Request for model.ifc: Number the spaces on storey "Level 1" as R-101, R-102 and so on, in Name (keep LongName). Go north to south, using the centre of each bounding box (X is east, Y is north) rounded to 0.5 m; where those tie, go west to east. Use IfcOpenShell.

First a look at what the model holds.

```python
import ifcopenshell
import ifcopenshell.util.element
import ifcopenshell.util.placement

model = ifcopenshell.open("model.ifc")
print(model.schema)
storey = next(s for s in model.by_type("IfcBuildingStorey") if s.Name == "Level 1")
spaces = [e for e in ifcopenshell.util.element.get_decomposition(storey) if e.is_a("IfcSpace")]
for e in sorted(spaces, key=lambda e: e.id()):
    origin = ifcopenshell.util.placement.get_local_placement(e.ObjectPlacement)[:3, 3]
    print(e.id(), e.Name, e.LongName, origin.round(2) + 0.0, sep=" | ")
```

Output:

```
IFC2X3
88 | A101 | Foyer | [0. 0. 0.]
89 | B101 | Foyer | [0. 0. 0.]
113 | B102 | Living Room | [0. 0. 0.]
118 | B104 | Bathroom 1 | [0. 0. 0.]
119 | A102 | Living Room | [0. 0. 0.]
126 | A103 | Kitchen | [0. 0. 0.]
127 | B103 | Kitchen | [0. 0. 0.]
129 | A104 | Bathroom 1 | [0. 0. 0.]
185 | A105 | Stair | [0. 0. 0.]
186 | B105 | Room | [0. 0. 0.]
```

```python
import ifcopenshell
import ifcopenshell.geom
import ifcopenshell.util.element
import ifcopenshell.util.shape

model = ifcopenshell.open("model.ifc")
settings = ifcopenshell.geom.settings()
settings.set("use-world-coords", True)


def centre(element):
    shape = ifcopenshell.geom.create_shape(settings, element)
    return ifcopenshell.util.shape.get_bbox_centroid(shape.geometry)


storey = next(s for s in model.by_type("IfcBuildingStorey") if s.Name == "Level 1")
spaces = [e for e in ifcopenshell.util.element.get_decomposition(storey) if e.is_a("IfcSpace")]

# Insertion points can sit at a corner or the storey origin, so sort by the geometry (in metres).
centres = {e: centre(e) for e in spaces}
spaces.sort(key=lambda e: (-round(centres[e][1] / 0.5), centres[e][0]))

for i, e in enumerate(spaces, start=1):
    number = f"R-1{i:02d}"
    e.Name = number
    print(e.id(), number)

model.write("model_rev.ifc")
```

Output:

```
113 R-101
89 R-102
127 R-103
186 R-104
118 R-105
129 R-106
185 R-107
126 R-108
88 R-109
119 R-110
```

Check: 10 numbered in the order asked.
